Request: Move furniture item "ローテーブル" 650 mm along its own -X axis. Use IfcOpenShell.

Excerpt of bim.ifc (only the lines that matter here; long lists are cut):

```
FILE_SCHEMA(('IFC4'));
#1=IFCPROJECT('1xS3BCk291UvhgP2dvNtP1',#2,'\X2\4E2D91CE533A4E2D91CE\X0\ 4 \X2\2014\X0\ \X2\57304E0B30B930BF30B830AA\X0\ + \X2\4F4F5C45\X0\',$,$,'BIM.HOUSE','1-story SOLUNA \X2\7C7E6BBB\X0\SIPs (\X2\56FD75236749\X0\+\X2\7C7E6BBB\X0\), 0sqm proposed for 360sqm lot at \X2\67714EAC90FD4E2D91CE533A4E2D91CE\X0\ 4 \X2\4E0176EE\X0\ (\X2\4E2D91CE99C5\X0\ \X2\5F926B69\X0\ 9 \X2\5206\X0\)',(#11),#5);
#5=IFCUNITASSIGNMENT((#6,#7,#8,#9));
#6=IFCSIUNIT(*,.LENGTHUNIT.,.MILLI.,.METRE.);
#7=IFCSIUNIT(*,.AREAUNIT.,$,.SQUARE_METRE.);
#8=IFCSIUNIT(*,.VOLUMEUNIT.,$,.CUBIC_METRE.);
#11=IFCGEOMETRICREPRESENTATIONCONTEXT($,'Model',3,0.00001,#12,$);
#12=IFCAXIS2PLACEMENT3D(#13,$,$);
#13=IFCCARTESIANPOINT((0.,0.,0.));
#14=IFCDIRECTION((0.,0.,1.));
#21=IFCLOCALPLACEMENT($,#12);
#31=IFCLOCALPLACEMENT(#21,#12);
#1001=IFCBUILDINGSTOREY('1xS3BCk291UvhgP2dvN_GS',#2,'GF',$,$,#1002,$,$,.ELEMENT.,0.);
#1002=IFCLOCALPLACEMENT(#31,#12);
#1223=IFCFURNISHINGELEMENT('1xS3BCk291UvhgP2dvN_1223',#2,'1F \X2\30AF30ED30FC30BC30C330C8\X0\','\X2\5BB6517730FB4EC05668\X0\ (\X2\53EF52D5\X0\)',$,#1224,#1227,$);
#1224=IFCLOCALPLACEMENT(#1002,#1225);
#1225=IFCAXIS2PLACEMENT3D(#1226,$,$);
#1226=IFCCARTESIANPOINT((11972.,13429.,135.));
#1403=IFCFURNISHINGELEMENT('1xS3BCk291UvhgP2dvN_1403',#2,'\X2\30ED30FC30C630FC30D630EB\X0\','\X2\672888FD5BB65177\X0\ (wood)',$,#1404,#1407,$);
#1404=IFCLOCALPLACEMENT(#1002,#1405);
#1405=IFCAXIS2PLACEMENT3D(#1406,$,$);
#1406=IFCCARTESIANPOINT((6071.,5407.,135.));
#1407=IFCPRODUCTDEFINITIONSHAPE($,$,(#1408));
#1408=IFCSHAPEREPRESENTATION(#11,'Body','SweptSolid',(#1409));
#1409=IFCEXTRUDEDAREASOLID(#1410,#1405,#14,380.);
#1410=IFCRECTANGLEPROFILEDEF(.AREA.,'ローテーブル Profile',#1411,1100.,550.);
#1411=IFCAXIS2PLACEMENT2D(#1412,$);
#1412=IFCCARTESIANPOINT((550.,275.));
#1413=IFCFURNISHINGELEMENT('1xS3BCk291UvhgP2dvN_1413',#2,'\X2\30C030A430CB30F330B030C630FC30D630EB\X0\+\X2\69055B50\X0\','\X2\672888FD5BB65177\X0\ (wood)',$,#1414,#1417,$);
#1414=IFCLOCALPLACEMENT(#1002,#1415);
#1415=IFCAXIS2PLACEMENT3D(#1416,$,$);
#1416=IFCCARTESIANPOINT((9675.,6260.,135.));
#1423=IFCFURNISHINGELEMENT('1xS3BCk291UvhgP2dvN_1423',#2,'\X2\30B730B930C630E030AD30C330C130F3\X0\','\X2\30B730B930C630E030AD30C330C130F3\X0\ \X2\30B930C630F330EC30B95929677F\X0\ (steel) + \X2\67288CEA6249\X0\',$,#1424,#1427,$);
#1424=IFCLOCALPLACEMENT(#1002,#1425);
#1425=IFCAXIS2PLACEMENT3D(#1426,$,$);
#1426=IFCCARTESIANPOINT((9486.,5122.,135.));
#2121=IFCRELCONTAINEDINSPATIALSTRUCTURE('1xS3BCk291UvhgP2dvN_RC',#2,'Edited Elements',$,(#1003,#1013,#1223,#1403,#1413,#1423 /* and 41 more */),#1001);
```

```python
import ifcopenshell
import ifcopenshell.api.geometry
import ifcopenshell.util.placement

model = ifcopenshell.open("bim.ifc")

item = model.by_guid("1xS3BCk291UvhgP2dvN_1403")
matrix = ifcopenshell.util.placement.get_local_placement(item.ObjectPlacement)
matrix[:3, 3] -= matrix[:3, 0] * 650.0
ifcopenshell.api.geometry.edit_object_placement(model, product=item, matrix=matrix, is_si=False)

print(ifcopenshell.util.placement.get_local_placement(item.ObjectPlacement).round(3) + 0.0)

model.write("bim_edited.ifc")
```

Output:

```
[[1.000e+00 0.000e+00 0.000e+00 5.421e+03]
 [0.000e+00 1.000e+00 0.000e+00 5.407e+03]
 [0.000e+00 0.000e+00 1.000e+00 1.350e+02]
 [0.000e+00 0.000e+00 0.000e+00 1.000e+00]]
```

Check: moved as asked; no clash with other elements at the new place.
